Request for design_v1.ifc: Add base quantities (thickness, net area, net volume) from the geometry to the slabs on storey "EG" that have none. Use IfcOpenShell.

First a look at what the model holds.

```python
import ifcopenshell
import ifcopenshell.util.element
import ifcopenshell.util.unit

model = ifcopenshell.open("design_v1.ifc")
print(model.schema)
for unit_type in ("LENGTHUNIT", "AREAUNIT", "VOLUMEUNIT"):
    print(unit_type, ifcopenshell.util.unit.calculate_unit_scale(model, unit_type))
storey = next(s for s in model.by_type("IfcBuildingStorey") if s.Name == "EG")
slabs = [e for e in ifcopenshell.util.element.get_decomposition(storey) if e.is_a("IfcSlab")]
for e in sorted(slabs, key=lambda e: e.id()):
    print(e.id(), e.is_a(), e.Name, list(ifcopenshell.util.element.get_psets(e, qtos_only=True)), sep=" | ")
```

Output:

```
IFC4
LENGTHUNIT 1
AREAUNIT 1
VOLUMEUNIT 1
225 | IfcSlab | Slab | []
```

```python
import ifcopenshell
import ifcopenshell.api.pset
import ifcopenshell.geom
import ifcopenshell.util.element
import ifcopenshell.util.shape
import ifcopenshell.util.unit

model = ifcopenshell.open("design_v1.ifc")
unit_scale = ifcopenshell.util.unit.calculate_unit_scale(model)
area_scale = ifcopenshell.util.unit.calculate_unit_scale(model, "AREAUNIT")
volume_scale = ifcopenshell.util.unit.calculate_unit_scale(model, "VOLUMEUNIT")
settings = ifcopenshell.geom.settings()

storey = next(s for s in model.by_type("IfcBuildingStorey") if s.Name == "EG")
slabs = [e for e in ifcopenshell.util.element.get_decomposition(storey) if e.is_a("IfcSlab")]

for e in sorted(slabs, key=lambda e: e.id()):
    if ifcopenshell.util.element.get_psets(e, qtos_only=True, should_inherit=False):
        continue
    # Geometry comes back in metres, in the element's own axes.
    shape = ifcopenshell.geom.create_shape(settings, e)
    values = {
        "Width": ifcopenshell.util.shape.get_z(shape.geometry) / unit_scale,
        "NetArea": ifcopenshell.util.shape.get_footprint_area(shape.geometry) / area_scale,
        "NetVolume": ifcopenshell.util.shape.get_volume(shape.geometry) / volume_scale,
    }
    qto = ifcopenshell.api.pset.add_qto(model, product=e, name="Qto_SlabBaseQuantities")
    ifcopenshell.api.pset.edit_qto(model, qto=qto, properties=values)
    print(e.id(), {k: round(v, 3) for k, v in values.items()})

model.write("design_v1_updated.ifc")
```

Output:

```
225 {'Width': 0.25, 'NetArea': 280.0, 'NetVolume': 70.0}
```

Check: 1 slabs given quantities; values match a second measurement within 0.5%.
